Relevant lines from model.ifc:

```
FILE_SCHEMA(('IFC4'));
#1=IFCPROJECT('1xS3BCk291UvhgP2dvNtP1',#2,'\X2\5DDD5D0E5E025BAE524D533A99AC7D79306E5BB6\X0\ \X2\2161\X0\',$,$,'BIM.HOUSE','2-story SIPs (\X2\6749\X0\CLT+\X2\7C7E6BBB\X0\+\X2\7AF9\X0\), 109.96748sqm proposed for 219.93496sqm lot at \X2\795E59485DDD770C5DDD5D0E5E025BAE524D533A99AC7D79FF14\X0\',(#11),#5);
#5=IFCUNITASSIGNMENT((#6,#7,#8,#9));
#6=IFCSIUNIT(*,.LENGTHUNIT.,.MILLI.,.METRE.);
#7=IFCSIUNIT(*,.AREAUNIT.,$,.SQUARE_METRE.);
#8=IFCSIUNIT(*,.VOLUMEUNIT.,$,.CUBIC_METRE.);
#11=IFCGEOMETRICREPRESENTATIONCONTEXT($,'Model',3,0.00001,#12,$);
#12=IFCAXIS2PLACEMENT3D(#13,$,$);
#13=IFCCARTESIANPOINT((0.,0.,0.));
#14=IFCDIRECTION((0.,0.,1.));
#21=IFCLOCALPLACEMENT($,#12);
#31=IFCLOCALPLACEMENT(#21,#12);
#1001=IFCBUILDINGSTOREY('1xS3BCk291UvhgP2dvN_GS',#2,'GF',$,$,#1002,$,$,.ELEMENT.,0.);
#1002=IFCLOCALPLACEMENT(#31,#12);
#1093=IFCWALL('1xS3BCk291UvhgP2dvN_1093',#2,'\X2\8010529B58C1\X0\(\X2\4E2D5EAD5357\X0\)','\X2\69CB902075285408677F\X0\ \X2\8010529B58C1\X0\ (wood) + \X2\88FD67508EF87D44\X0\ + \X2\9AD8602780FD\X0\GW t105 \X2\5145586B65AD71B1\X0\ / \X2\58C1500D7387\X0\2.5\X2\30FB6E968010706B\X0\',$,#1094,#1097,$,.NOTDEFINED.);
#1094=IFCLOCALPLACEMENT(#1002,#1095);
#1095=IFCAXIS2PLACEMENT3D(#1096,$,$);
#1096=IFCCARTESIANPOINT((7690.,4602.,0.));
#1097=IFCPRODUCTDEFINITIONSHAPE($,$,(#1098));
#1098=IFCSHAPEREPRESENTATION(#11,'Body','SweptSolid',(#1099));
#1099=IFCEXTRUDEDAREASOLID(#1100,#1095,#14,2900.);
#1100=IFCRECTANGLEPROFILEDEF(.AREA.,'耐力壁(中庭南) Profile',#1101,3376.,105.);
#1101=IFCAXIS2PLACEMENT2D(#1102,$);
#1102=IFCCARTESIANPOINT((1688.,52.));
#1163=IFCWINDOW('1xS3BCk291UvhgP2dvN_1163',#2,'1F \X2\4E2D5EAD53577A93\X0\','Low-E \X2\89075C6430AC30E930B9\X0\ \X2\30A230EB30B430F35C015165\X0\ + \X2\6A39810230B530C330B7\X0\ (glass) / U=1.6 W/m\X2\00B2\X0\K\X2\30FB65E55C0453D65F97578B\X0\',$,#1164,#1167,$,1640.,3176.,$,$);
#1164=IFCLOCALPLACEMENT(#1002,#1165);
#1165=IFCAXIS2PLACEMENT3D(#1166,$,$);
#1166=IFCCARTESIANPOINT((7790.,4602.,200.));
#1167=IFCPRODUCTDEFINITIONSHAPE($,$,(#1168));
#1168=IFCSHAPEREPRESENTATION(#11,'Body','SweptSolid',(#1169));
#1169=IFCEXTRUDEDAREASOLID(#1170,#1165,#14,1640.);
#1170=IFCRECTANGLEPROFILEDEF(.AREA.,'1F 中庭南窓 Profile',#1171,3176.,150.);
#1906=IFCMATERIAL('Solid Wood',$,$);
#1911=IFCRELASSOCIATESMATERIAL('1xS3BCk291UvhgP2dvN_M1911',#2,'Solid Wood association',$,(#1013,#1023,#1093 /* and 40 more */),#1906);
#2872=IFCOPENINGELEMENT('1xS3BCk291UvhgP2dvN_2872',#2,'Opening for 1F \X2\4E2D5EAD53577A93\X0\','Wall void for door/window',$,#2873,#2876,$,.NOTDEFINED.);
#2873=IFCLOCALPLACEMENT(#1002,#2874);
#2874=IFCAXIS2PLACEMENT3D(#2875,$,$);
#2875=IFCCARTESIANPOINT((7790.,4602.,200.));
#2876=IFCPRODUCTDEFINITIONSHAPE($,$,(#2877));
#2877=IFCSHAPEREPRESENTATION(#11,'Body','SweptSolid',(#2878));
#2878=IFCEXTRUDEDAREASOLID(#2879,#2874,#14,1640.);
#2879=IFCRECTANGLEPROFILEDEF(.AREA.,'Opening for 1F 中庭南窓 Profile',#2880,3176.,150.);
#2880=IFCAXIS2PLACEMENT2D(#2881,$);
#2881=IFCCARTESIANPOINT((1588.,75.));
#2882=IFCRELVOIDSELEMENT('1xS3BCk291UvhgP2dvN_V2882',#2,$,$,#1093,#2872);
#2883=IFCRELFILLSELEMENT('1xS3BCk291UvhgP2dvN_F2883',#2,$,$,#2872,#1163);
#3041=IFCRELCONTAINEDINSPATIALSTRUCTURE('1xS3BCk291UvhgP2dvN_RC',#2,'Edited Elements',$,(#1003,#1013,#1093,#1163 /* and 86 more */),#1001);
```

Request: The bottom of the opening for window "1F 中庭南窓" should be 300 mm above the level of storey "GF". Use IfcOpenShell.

```python
import numpy as np
import ifcopenshell
import ifcopenshell.api.geometry
import ifcopenshell.geom
import ifcopenshell.util.element
import ifcopenshell.util.placement
import ifcopenshell.util.shape
import ifcopenshell.util.unit

model = ifcopenshell.open("model.ifc")
unit_scale = ifcopenshell.util.unit.calculate_unit_scale(model)

window = model.by_id(1163)
opening = window.FillsVoids[0].RelatingOpeningElement
storey = ifcopenshell.util.element.get_container(window, ifc_class="IfcBuildingStorey")
level = ifcopenshell.util.placement.get_local_placement(storey.ObjectPlacement)[2, 3]

# The opening's origin need not be at the sill, so measure its lowest point.
shape = ifcopenshell.geom.create_shape(ifcopenshell.geom.settings(), opening)
bottom = ifcopenshell.util.shape.get_shape_bottom_elevation(shape, shape.geometry) / unit_scale
dz = level + 300.0 - bottom

shift = np.array([0.0, 0.0, dz])
# The window is not placed relative to its opening, so move both.
for product in (opening, window):
    matrix = ifcopenshell.util.placement.get_local_placement(product.ObjectPlacement)
    matrix[:3, 3] += shift
    ifcopenshell.api.geometry.edit_object_placement(model, product=product, matrix=matrix, is_si=False)

print(f"moved by {dz * unit_scale:+.3f} m")

model.write("model_rev.ifc")
```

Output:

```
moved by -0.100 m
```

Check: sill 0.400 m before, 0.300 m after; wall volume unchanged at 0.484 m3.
